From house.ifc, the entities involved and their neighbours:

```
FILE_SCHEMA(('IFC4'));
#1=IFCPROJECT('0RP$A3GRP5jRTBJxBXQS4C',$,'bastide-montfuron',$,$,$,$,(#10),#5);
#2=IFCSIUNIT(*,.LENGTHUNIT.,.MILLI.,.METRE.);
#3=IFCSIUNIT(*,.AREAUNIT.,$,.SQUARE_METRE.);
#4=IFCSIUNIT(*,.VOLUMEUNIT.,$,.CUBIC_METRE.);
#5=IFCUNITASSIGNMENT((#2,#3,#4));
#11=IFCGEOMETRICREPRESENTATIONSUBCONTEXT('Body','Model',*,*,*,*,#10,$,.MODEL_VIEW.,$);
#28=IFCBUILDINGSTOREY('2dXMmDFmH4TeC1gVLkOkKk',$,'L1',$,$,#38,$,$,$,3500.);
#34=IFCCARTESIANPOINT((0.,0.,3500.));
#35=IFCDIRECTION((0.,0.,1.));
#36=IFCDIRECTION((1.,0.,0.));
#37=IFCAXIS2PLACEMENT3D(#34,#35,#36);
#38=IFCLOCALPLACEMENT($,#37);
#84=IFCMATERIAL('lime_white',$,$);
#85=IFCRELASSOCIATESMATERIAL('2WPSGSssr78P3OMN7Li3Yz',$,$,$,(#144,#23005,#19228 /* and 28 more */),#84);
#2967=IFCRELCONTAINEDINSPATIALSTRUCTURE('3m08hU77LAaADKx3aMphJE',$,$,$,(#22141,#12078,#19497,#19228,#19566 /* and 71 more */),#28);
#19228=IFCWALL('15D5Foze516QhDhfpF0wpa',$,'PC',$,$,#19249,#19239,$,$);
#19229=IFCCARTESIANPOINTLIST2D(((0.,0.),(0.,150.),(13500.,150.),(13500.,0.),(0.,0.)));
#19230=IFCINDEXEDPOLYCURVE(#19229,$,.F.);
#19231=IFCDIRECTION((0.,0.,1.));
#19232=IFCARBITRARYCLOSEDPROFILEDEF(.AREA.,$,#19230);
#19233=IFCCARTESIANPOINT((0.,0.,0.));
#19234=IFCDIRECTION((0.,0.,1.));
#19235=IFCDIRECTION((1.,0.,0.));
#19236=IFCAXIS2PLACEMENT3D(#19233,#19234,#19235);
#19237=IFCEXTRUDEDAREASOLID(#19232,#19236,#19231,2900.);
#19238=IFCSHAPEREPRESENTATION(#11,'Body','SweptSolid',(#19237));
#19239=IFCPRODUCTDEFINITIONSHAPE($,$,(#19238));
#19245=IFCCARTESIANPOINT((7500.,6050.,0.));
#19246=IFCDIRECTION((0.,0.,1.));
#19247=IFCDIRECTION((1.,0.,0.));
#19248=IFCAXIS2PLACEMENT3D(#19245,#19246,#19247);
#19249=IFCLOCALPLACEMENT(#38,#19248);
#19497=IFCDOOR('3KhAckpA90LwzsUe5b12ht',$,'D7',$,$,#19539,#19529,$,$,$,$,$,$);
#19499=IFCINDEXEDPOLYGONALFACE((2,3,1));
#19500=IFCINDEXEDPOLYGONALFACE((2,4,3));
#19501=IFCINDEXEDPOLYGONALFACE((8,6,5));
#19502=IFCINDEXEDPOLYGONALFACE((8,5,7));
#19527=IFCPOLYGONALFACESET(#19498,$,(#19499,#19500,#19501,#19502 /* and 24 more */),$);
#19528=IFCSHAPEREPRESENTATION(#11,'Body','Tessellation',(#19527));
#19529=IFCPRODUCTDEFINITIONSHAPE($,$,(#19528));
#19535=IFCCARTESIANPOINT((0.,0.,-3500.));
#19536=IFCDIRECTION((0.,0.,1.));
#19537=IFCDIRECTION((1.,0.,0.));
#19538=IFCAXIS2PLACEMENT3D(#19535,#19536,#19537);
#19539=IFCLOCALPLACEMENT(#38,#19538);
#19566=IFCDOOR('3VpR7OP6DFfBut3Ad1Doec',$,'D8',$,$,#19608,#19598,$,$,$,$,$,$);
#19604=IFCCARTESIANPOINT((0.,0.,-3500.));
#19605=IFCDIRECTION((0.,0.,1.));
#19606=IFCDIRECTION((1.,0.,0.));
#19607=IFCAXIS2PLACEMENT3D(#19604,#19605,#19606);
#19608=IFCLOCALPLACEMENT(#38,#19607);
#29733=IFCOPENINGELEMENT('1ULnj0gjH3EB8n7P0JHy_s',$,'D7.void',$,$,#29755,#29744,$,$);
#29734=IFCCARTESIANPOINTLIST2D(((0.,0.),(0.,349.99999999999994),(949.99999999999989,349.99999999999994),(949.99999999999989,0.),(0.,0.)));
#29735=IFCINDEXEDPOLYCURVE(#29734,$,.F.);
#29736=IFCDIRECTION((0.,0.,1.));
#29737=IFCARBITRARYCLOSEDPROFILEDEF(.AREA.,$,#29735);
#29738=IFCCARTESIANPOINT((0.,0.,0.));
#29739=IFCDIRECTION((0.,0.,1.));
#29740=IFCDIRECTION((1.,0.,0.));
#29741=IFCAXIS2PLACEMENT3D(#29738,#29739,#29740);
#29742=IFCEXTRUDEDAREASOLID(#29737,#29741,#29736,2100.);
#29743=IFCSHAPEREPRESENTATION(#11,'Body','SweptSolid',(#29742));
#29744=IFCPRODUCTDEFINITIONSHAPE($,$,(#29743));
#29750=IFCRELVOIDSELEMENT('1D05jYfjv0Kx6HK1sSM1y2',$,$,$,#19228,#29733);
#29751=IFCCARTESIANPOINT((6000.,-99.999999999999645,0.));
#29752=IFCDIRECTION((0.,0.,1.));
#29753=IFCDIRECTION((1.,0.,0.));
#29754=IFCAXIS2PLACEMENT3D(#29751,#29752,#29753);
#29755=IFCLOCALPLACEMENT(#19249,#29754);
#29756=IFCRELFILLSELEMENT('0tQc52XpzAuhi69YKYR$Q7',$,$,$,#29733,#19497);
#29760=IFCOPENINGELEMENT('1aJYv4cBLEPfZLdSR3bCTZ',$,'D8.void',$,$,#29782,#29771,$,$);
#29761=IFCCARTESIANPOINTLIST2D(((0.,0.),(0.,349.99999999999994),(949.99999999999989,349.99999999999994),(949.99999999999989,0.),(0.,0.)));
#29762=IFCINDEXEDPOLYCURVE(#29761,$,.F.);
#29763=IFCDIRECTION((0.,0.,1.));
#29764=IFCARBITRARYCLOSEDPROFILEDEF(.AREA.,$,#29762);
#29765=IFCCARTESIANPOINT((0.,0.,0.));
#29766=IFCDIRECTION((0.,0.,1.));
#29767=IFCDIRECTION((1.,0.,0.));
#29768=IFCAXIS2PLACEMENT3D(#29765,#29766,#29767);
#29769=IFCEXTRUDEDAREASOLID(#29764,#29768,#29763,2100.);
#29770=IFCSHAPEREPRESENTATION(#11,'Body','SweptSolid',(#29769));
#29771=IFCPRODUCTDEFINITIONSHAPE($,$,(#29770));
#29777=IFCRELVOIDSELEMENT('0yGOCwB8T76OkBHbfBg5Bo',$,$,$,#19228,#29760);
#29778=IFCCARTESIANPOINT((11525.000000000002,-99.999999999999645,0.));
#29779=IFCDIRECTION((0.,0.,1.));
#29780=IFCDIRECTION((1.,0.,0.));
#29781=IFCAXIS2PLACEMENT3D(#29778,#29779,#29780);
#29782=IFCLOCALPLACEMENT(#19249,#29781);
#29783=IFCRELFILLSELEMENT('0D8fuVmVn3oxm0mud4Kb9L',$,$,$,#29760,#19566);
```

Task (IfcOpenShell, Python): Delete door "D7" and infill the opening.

```python
import ifcopenshell
import ifcopenshell.api.feature
import ifcopenshell.api.root
import ifcopenshell.geom
import ifcopenshell.util.shape

model = ifcopenshell.open("house.ifc")
settings = ifcopenshell.geom.settings()


def volume(element):
    """Net volume in cubic metres, openings subtracted."""
    shape = ifcopenshell.geom.create_shape(settings, element)
    return ifcopenshell.util.shape.get_volume(shape.geometry)


door = model.by_guid("3KhAckpA90LwzsUe5b12ht")
opening = door.FillsVoids[0].RelatingOpeningElement
wall = opening.VoidsElements[0].RelatingBuildingElement
before = volume(wall)

ifcopenshell.api.root.remove_product(model, product=door)
ifcopenshell.api.feature.remove_feature(model, feature=opening)

after = volume(wall)

print(f"wall volume {before:.3f} -> {after:.3f} m3")

model.write("house_rev.ifc")
```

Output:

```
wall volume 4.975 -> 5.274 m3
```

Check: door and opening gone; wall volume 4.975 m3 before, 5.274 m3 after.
